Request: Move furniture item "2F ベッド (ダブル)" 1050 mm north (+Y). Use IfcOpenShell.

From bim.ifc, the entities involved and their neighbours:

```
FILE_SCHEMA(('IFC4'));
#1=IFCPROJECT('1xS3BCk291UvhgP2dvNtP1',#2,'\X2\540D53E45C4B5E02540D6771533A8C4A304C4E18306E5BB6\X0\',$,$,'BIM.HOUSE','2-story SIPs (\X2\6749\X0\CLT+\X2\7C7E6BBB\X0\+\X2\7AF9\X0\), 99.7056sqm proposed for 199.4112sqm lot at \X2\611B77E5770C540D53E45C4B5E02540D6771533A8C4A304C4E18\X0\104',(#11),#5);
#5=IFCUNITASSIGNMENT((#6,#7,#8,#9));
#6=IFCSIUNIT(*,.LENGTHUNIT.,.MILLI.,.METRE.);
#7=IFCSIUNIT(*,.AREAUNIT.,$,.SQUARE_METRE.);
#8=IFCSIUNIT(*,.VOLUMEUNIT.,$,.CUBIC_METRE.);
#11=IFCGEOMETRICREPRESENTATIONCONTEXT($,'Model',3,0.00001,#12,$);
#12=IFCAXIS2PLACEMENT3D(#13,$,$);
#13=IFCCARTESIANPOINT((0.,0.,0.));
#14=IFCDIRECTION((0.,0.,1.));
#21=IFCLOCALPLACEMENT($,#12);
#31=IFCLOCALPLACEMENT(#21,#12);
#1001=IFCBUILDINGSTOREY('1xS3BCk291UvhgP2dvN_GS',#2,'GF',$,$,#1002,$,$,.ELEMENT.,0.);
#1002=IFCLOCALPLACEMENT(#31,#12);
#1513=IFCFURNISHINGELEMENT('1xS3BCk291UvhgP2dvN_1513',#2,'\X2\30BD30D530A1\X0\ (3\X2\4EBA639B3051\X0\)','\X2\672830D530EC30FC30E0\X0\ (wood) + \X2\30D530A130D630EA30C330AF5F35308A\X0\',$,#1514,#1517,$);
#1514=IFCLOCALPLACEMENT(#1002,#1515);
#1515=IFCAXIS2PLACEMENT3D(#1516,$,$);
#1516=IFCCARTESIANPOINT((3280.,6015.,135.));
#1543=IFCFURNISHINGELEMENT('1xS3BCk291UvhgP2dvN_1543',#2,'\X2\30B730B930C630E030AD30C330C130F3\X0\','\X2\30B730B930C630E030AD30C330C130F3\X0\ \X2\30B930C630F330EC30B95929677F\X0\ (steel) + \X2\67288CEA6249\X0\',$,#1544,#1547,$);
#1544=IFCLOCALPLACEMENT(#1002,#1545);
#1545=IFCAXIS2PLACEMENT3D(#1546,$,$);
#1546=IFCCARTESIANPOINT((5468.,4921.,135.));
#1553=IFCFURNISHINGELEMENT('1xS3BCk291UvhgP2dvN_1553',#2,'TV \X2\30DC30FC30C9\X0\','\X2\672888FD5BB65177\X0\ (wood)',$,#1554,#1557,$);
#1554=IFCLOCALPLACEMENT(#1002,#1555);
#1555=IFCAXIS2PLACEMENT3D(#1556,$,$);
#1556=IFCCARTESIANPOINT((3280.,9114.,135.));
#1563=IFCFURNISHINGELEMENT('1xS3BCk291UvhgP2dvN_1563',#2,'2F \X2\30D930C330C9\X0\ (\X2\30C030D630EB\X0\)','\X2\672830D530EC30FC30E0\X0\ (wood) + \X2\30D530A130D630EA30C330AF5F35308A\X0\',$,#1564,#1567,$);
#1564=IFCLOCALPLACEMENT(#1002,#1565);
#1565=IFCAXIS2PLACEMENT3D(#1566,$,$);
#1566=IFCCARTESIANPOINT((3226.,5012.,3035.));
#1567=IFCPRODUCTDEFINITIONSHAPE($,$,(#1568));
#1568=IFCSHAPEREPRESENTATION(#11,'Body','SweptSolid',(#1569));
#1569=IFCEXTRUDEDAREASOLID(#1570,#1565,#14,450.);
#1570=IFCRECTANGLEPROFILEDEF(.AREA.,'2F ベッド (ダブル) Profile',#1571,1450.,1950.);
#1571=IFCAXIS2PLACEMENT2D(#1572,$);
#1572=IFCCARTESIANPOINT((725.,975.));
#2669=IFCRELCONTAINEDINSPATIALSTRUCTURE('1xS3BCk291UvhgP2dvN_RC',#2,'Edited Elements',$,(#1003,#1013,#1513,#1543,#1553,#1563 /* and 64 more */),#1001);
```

```python
import ifcopenshell
import ifcopenshell.api.geometry
import ifcopenshell.util.placement
import ifcopenshell.util.unit

model = ifcopenshell.open("bim.ifc")
unit_scale = ifcopenshell.util.unit.calculate_unit_scale(model)

item = model.by_guid("1xS3BCk291UvhgP2dvN_1563")
matrix = ifcopenshell.util.placement.get_local_placement(item.ObjectPlacement)
matrix[1, 3] += 1.05 / unit_scale
ifcopenshell.api.geometry.edit_object_placement(model, product=item, matrix=matrix, is_si=False)

print(ifcopenshell.util.placement.get_local_placement(item.ObjectPlacement).round(3) + 0.0)

model.write("bim-out.ifc")
```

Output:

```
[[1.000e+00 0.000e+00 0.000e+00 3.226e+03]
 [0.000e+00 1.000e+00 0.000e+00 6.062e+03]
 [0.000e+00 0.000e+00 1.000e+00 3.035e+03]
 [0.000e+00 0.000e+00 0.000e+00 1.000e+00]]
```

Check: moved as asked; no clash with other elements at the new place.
